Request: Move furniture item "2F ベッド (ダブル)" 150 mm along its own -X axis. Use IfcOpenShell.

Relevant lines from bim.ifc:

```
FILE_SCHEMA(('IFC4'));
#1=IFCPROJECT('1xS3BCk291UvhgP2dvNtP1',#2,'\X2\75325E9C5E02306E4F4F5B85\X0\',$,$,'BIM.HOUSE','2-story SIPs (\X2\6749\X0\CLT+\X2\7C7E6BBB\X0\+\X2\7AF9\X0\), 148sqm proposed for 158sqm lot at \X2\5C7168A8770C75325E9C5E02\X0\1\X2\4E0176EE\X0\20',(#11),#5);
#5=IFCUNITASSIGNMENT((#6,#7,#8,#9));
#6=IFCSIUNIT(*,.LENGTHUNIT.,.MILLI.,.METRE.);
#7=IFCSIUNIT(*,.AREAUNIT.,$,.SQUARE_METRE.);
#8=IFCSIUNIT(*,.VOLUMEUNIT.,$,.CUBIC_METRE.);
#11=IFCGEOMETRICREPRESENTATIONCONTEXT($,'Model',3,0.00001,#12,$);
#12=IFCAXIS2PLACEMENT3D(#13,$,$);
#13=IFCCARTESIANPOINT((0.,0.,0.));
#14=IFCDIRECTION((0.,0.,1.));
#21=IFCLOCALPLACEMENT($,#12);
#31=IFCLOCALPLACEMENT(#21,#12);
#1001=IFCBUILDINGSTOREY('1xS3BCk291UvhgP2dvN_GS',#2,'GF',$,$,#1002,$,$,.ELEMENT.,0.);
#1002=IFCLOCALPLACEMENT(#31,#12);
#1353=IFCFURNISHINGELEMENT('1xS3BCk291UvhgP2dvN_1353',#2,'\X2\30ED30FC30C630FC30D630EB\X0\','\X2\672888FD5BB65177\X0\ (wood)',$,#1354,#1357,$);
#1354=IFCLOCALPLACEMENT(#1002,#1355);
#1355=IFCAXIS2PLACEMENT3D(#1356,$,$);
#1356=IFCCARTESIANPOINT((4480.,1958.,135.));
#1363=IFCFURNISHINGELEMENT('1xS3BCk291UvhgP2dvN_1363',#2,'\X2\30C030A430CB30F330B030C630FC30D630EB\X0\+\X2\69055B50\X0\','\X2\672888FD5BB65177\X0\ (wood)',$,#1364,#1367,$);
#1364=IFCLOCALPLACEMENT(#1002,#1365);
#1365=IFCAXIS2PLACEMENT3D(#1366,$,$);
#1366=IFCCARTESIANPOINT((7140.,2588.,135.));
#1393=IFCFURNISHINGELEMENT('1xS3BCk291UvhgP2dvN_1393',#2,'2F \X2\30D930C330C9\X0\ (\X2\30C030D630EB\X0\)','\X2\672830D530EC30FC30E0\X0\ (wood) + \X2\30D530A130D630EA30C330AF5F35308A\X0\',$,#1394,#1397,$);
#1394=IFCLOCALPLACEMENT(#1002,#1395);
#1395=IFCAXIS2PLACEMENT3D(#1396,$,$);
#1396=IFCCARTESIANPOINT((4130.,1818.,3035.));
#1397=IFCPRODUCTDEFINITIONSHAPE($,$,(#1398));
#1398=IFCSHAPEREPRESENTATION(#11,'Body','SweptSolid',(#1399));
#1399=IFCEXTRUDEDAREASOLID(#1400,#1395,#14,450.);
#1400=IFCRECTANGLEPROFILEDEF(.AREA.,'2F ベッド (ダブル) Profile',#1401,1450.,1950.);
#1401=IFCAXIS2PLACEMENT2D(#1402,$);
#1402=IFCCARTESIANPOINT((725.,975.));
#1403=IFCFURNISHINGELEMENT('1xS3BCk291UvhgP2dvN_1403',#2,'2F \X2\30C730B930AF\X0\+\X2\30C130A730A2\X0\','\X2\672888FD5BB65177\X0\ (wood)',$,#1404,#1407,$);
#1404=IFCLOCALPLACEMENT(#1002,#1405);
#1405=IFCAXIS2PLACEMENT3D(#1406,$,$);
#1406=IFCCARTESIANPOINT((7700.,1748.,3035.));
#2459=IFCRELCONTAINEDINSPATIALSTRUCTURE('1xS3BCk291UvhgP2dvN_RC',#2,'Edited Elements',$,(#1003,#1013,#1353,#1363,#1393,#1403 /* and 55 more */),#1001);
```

```python
import ifcopenshell
import ifcopenshell.api.geometry
import ifcopenshell.util.placement

model = ifcopenshell.open("bim.ifc")

item = model.by_guid("1xS3BCk291UvhgP2dvN_1393")
matrix = ifcopenshell.util.placement.get_local_placement(item.ObjectPlacement)
matrix[:3, 3] -= matrix[:3, 0] * 150.0
ifcopenshell.api.geometry.edit_object_placement(model, product=item, matrix=matrix, is_si=False)

print(ifcopenshell.util.placement.get_local_placement(item.ObjectPlacement).round(3) + 0.0)

model.write("bim_edited.ifc")
```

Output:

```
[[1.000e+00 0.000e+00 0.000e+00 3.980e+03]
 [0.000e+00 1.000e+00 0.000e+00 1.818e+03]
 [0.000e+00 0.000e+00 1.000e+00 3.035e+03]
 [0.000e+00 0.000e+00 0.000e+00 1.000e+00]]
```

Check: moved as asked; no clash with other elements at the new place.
